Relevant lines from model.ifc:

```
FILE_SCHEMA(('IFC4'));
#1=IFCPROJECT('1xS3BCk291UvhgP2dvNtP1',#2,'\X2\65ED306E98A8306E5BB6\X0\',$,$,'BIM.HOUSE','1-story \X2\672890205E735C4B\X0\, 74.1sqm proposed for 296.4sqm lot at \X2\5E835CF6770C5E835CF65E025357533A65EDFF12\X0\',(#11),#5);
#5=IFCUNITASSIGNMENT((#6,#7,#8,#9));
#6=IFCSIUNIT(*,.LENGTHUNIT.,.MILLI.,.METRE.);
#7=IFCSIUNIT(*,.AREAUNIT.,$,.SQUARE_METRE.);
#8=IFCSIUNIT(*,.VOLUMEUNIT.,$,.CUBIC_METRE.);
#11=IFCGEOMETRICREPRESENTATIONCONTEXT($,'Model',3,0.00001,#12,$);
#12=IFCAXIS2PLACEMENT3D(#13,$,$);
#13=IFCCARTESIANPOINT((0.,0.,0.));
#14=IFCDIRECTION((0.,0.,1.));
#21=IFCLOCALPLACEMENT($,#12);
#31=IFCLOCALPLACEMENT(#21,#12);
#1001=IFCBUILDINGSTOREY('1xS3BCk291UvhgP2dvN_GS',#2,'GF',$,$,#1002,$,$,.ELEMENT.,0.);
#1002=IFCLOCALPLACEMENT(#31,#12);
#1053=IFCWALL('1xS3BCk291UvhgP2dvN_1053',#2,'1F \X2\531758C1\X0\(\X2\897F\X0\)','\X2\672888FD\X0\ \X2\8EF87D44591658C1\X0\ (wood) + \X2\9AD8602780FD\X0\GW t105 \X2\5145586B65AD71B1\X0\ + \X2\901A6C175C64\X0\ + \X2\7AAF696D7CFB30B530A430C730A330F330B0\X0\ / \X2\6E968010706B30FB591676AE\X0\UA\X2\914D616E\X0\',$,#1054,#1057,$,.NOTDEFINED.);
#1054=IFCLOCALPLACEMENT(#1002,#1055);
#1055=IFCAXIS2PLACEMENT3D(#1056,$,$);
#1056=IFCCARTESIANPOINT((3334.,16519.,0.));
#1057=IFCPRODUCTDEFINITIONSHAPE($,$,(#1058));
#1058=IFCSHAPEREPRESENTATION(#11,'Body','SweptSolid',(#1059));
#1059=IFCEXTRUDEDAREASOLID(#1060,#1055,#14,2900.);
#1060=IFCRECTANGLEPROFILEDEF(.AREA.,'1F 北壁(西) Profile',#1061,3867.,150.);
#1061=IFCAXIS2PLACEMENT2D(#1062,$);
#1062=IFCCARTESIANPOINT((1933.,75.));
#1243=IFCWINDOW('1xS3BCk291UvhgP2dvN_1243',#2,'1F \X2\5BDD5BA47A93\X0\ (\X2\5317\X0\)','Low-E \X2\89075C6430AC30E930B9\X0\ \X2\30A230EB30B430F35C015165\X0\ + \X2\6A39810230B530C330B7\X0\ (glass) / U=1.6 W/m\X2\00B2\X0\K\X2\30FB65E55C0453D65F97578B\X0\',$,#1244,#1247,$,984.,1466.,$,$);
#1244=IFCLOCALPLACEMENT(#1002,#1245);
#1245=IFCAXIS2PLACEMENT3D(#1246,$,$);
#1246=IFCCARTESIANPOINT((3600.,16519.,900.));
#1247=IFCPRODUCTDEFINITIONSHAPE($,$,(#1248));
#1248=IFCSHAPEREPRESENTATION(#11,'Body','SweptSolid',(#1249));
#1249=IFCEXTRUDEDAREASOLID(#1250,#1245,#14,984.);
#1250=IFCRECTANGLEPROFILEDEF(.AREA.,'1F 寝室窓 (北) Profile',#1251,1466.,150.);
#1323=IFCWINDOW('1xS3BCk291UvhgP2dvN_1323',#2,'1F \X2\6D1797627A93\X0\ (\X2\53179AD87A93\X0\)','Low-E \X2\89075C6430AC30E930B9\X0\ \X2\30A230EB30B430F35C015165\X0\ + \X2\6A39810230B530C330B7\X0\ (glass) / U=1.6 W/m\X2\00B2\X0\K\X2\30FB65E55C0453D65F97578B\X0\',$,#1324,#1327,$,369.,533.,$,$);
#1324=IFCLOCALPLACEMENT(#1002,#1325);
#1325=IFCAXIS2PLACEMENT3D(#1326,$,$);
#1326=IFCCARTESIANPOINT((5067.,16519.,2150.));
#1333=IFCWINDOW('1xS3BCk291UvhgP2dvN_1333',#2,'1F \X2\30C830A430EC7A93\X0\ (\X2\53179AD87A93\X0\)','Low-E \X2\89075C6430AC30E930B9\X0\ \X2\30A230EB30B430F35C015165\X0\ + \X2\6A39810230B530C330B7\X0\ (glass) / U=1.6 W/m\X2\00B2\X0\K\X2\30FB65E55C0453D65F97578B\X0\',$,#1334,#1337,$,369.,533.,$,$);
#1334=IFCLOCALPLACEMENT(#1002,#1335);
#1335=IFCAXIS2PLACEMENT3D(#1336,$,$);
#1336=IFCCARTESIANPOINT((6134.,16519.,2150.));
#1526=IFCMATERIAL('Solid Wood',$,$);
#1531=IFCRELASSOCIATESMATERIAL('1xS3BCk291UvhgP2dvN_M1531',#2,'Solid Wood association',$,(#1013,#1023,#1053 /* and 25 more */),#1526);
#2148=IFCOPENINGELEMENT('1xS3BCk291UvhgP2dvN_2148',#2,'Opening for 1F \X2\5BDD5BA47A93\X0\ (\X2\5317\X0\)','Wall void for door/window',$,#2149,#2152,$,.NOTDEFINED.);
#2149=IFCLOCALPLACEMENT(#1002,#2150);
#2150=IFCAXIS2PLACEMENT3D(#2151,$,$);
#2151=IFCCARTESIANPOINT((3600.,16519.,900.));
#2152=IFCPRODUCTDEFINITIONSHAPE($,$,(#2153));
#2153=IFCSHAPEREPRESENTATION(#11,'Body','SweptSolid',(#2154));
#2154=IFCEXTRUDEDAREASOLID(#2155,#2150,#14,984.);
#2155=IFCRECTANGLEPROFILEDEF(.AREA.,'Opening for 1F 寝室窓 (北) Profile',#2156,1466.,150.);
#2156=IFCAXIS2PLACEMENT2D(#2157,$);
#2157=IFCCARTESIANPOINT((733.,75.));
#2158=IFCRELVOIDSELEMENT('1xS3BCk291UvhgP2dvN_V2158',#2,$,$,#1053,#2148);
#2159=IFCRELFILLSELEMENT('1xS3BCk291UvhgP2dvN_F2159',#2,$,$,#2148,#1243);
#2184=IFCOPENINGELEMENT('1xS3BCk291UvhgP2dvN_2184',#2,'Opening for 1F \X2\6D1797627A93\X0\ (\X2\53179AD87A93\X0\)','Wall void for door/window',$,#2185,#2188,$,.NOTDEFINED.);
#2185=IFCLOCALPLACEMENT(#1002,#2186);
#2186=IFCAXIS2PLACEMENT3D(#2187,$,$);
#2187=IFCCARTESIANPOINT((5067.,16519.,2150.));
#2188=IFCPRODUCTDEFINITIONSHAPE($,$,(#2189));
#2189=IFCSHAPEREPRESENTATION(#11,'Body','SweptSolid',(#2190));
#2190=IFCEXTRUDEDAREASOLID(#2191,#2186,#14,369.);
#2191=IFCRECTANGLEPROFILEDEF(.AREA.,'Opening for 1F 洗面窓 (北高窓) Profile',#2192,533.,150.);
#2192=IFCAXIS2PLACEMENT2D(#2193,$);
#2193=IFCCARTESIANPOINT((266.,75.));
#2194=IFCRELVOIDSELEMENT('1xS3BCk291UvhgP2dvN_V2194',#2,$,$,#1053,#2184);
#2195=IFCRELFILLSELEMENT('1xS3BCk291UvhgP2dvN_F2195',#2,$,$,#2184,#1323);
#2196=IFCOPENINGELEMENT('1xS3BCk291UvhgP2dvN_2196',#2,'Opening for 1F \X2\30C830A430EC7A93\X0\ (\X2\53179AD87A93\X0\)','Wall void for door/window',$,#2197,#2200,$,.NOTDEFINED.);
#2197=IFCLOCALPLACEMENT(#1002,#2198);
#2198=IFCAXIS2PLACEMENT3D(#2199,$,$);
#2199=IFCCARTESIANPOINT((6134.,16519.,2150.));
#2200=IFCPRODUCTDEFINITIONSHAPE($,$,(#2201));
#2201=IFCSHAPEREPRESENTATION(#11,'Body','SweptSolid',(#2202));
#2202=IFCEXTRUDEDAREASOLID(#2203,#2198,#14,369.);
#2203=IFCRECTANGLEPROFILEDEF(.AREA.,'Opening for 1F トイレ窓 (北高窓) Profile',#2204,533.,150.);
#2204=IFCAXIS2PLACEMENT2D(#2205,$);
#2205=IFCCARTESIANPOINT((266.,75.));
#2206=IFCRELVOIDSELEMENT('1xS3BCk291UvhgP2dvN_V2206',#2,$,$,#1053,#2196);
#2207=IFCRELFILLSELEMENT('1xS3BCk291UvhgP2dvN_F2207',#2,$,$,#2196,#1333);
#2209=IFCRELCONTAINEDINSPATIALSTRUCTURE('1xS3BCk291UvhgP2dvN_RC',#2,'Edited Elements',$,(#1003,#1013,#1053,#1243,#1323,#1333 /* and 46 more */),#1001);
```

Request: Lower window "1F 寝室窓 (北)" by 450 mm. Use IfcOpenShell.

```python
import numpy as np
import ifcopenshell
import ifcopenshell.api.geometry
import ifcopenshell.util.placement
import ifcopenshell.util.unit

model = ifcopenshell.open("model.ifc")
unit_scale = ifcopenshell.util.unit.calculate_unit_scale(model)

window = model.by_guid("1xS3BCk291UvhgP2dvN_1243")
opening = window.FillsVoids[0].RelatingOpeningElement
dz = -450.0

shift = np.array([0.0, 0.0, dz])
# The window is not placed relative to its opening, so move both.
for product in (opening, window):
    matrix = ifcopenshell.util.placement.get_local_placement(product.ObjectPlacement)
    matrix[:3, 3] += shift
    ifcopenshell.api.geometry.edit_object_placement(model, product=product, matrix=matrix, is_si=False)

print(f"moved by {dz * unit_scale:+.3f} m")

model.write("model_updated.ifc")
```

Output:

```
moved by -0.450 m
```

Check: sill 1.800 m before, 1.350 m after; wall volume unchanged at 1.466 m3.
